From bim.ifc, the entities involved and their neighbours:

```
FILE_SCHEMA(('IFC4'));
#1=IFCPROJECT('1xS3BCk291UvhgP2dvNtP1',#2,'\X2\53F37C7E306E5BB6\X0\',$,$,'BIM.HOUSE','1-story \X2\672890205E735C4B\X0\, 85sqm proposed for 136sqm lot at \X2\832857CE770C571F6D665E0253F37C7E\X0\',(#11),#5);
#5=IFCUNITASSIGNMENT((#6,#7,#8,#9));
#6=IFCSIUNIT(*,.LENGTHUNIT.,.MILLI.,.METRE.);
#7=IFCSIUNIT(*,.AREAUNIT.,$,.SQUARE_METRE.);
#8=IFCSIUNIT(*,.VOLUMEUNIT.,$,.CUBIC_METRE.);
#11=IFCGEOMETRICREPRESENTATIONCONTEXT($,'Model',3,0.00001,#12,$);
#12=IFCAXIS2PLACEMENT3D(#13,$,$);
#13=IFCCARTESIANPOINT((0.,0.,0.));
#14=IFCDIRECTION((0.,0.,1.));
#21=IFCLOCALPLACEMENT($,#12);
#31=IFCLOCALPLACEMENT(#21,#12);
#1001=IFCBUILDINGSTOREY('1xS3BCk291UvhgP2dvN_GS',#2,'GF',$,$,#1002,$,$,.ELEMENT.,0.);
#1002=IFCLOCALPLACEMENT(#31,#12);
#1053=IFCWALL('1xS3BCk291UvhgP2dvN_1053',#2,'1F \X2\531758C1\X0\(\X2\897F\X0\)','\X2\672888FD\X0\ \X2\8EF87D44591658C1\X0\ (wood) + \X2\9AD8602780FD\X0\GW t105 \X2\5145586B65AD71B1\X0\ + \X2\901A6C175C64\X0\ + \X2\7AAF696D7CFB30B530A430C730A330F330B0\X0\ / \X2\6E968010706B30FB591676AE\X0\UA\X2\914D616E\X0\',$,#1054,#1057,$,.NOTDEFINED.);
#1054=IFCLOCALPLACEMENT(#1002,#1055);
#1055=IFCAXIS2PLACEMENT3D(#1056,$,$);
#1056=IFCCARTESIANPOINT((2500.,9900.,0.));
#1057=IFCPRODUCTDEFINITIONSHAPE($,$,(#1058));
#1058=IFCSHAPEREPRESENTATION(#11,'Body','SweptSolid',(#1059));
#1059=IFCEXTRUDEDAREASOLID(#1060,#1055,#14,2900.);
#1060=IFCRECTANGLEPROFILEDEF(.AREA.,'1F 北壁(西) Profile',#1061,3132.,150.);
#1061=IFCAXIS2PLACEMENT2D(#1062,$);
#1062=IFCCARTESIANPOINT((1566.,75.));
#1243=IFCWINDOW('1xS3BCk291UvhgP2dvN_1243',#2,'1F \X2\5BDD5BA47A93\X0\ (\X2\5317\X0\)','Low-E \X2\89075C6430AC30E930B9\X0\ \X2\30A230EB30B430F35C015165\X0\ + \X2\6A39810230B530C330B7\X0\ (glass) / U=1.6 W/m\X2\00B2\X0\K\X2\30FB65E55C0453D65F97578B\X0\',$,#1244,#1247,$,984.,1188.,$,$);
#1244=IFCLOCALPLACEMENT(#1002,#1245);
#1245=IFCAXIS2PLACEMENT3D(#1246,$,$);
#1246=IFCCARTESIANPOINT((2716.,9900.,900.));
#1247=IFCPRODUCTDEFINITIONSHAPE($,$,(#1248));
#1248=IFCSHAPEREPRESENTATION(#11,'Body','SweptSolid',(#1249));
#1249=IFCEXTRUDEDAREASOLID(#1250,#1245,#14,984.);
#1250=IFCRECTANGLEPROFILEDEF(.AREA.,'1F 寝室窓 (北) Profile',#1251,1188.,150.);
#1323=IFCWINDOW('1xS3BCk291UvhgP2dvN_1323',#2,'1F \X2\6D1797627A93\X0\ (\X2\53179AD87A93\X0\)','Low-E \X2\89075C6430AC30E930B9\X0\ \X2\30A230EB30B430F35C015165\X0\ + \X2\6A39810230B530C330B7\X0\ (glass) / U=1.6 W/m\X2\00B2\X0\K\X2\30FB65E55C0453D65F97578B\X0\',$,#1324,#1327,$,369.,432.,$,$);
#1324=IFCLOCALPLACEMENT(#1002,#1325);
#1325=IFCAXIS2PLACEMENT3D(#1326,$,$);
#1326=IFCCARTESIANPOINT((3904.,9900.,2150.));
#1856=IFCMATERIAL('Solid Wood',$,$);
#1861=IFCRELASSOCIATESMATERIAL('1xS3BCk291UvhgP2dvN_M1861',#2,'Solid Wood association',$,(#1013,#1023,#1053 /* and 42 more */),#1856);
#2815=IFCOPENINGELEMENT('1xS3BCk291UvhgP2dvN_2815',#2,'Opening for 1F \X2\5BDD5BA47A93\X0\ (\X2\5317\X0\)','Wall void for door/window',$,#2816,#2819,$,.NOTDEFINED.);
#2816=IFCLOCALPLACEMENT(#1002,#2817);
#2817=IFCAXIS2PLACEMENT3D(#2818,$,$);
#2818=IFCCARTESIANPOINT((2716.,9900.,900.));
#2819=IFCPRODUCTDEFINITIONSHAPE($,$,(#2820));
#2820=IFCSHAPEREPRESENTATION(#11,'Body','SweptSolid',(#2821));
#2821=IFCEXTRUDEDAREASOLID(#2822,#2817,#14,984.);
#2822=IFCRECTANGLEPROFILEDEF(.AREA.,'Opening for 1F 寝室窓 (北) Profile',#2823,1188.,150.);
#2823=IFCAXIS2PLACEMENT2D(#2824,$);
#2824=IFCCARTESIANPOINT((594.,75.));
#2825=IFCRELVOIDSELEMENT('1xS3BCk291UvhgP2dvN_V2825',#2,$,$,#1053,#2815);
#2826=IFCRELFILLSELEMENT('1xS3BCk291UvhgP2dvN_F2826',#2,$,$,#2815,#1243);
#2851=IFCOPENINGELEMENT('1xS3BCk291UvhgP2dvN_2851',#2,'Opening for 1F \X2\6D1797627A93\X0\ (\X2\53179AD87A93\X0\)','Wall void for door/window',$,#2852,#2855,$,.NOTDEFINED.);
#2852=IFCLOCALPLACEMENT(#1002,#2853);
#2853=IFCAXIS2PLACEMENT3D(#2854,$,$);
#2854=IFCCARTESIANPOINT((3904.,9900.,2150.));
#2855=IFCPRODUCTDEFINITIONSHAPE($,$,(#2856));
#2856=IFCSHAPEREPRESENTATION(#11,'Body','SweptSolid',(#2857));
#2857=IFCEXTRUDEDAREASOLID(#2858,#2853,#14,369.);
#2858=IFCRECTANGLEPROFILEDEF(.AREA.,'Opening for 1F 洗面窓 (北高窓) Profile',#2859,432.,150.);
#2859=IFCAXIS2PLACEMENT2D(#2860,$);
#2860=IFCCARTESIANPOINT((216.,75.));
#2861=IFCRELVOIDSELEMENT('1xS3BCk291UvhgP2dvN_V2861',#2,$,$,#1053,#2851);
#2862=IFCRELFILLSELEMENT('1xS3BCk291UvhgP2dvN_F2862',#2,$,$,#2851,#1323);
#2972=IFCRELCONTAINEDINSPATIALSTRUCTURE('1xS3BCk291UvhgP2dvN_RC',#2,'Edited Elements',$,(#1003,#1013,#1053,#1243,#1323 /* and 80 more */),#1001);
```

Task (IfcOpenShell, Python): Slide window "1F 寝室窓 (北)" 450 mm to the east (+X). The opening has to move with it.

```python
import ifcopenshell
import ifcopenshell.api.geometry
import ifcopenshell.util.placement

model = ifcopenshell.open("bim.ifc")

window = model.by_id(1243)
opening = window.FillsVoids[0].RelatingOpeningElement
wall = opening.VoidsElements[0].RelatingBuildingElement

wall_matrix = ifcopenshell.util.placement.get_local_placement(wall.ObjectPlacement)
shift = wall_matrix[:3, 0] * 450.0
before = ifcopenshell.util.placement.get_local_placement(window.ObjectPlacement)[:3, 3].copy()

# The window is not placed relative to its opening, so move both.
for product in (opening, window):
    matrix = ifcopenshell.util.placement.get_local_placement(product.ObjectPlacement)
    matrix[:3, 3] += shift
    ifcopenshell.api.geometry.edit_object_placement(model, product=product, matrix=matrix, is_si=False)

after = ifcopenshell.util.placement.get_local_placement(window.ObjectPlacement)[:3, 3]
print("window moved by", (after - before).round(3) + 0.0)

model.write("bim_updated.ifc")
```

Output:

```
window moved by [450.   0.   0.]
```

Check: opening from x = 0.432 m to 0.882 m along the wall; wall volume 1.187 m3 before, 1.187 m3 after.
